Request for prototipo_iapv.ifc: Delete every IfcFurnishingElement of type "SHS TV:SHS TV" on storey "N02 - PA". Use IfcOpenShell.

First a look at what the model holds.

```python
import ifcopenshell
import ifcopenshell.util.element

model = ifcopenshell.open("prototipo_iapv.ifc")
print(model.schema)
storey = next(s for s in model.by_type("IfcBuildingStorey") if s.Name == "N02 - PA")
furniture = [e for e in ifcopenshell.util.element.get_decomposition(storey) if e.is_a("IfcFurnishingElement")]
seen = {}
for e in furniture:
    element_type = ifcopenshell.util.element.get_type(e)
    name = element_type.Name if element_type not in (None, e) else None
    seen[name] = seen.get(name, 0) + 1
for name, count in sorted(seen.items(), key=str):
    print(count, "x", name)
```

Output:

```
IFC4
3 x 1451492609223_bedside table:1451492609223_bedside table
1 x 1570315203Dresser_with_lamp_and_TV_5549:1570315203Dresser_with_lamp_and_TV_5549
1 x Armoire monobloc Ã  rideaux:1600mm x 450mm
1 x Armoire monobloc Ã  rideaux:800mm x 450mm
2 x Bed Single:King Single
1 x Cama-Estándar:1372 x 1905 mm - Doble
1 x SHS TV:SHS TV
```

```python
import ifcopenshell
import ifcopenshell.api.root
import ifcopenshell.util.element

model = ifcopenshell.open("prototipo_iapv.ifc")

storey = next(s for s in model.by_type("IfcBuildingStorey") if s.Name == "N02 - PA")
furniture = [e for e in ifcopenshell.util.element.get_decomposition(storey) if e.is_a("IfcFurnishingElement")]
targets = [e for e in furniture if (t := ifcopenshell.util.element.get_type(e)) not in (None, e) and t.Name == "SHS TV:SHS TV"]

for e in targets:
    ifcopenshell.api.root.remove_product(model, product=e)
print(len(targets), "removed")

model.write("prototipo_iapv_edited.ifc")
```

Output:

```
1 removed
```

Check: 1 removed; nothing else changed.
